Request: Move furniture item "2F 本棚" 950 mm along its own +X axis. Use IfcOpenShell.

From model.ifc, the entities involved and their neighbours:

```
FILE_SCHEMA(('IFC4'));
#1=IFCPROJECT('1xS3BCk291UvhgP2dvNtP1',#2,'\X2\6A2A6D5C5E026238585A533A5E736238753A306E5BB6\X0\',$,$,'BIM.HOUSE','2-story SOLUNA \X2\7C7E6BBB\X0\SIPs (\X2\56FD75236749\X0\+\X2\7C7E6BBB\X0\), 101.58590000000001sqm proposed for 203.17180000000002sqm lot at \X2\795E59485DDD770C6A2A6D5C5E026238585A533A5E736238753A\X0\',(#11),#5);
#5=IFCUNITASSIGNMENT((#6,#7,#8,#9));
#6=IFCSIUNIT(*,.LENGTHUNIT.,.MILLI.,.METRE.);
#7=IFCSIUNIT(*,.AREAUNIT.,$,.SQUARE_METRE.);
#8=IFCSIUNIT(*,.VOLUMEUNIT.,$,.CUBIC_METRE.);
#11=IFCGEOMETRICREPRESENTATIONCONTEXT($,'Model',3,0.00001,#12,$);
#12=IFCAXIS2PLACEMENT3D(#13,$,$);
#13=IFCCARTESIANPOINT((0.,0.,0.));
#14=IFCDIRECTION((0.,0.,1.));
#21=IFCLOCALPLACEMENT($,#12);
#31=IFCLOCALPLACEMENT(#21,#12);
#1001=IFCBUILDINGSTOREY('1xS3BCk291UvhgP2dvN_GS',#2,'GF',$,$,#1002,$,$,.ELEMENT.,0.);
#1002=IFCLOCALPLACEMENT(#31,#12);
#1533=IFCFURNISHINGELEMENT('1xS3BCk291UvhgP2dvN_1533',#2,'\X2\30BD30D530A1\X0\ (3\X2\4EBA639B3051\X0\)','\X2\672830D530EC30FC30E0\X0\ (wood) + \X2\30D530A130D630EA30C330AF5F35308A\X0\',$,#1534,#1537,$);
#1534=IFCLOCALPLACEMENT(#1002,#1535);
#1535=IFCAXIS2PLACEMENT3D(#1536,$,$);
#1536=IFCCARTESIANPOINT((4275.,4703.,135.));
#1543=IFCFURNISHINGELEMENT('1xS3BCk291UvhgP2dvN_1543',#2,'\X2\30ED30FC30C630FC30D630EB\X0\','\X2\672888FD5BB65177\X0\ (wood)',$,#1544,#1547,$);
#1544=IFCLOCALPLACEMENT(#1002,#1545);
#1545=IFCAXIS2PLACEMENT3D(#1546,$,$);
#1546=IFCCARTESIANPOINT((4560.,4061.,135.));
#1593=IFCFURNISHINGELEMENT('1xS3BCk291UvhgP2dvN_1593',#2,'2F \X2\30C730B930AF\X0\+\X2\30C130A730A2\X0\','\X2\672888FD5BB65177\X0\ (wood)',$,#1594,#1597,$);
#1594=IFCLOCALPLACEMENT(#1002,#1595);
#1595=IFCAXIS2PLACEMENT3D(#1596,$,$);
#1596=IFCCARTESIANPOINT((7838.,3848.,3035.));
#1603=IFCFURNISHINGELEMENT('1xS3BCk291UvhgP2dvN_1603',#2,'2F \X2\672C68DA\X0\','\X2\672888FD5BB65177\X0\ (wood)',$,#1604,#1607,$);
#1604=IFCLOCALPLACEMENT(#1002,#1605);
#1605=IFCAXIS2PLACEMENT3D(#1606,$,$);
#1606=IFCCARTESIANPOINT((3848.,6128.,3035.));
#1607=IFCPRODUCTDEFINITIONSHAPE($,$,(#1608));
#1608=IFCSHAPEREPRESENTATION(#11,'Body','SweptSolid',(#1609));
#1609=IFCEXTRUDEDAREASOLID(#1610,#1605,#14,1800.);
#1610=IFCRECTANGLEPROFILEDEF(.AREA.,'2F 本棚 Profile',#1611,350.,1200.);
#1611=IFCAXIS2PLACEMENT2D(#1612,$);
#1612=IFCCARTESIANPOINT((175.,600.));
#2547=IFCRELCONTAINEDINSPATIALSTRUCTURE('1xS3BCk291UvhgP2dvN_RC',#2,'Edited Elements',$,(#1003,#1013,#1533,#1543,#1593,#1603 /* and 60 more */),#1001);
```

```python
import ifcopenshell
import ifcopenshell.api.geometry
import ifcopenshell.util.placement

model = ifcopenshell.open("model.ifc")

item = model.by_id(1603)
matrix = ifcopenshell.util.placement.get_local_placement(item.ObjectPlacement)
matrix[:3, 3] += matrix[:3, 0] * 950.0
ifcopenshell.api.geometry.edit_object_placement(model, product=item, matrix=matrix, is_si=False)

print(ifcopenshell.util.placement.get_local_placement(item.ObjectPlacement).round(3) + 0.0)

model.write("model-out.ifc")
```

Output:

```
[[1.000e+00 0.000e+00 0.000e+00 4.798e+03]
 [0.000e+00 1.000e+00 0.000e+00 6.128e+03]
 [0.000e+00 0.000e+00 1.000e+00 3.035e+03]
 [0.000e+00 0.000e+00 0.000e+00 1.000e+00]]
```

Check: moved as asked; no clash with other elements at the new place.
